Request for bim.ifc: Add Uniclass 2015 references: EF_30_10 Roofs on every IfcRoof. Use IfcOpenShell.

First a look at what the model holds.

```python
import ifcopenshell

model = ifcopenshell.open("bim.ifc")
print(model.schema)
print("classifications:", [c.Name for c in model.by_type("IfcClassification")])
for ifc_class in ("IfcDoor", "IfcRoof", "IfcStair", "IfcWall", "IfcWindow"):
    print(ifc_class, len(model.by_type(ifc_class)))
```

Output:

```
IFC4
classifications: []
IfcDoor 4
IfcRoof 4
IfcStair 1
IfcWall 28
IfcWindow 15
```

```python
import ifcopenshell
import ifcopenshell.api.classification

model = ifcopenshell.open("bim.ifc")

system = ifcopenshell.api.classification.add_classification(model, classification="Uniclass 2015")

codes = {
    "IfcRoof": ("EF_30_10", "Roofs"),
}
for ifc_class, (code, name) in codes.items():
    products = model.by_type(ifc_class)
    ifcopenshell.api.classification.add_reference(
        model, products=products, classification=system, identification=code, name=name
    )
    print(code, len(products))

model.write("bim_v2.ifc")
```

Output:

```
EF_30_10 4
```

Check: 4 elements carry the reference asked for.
